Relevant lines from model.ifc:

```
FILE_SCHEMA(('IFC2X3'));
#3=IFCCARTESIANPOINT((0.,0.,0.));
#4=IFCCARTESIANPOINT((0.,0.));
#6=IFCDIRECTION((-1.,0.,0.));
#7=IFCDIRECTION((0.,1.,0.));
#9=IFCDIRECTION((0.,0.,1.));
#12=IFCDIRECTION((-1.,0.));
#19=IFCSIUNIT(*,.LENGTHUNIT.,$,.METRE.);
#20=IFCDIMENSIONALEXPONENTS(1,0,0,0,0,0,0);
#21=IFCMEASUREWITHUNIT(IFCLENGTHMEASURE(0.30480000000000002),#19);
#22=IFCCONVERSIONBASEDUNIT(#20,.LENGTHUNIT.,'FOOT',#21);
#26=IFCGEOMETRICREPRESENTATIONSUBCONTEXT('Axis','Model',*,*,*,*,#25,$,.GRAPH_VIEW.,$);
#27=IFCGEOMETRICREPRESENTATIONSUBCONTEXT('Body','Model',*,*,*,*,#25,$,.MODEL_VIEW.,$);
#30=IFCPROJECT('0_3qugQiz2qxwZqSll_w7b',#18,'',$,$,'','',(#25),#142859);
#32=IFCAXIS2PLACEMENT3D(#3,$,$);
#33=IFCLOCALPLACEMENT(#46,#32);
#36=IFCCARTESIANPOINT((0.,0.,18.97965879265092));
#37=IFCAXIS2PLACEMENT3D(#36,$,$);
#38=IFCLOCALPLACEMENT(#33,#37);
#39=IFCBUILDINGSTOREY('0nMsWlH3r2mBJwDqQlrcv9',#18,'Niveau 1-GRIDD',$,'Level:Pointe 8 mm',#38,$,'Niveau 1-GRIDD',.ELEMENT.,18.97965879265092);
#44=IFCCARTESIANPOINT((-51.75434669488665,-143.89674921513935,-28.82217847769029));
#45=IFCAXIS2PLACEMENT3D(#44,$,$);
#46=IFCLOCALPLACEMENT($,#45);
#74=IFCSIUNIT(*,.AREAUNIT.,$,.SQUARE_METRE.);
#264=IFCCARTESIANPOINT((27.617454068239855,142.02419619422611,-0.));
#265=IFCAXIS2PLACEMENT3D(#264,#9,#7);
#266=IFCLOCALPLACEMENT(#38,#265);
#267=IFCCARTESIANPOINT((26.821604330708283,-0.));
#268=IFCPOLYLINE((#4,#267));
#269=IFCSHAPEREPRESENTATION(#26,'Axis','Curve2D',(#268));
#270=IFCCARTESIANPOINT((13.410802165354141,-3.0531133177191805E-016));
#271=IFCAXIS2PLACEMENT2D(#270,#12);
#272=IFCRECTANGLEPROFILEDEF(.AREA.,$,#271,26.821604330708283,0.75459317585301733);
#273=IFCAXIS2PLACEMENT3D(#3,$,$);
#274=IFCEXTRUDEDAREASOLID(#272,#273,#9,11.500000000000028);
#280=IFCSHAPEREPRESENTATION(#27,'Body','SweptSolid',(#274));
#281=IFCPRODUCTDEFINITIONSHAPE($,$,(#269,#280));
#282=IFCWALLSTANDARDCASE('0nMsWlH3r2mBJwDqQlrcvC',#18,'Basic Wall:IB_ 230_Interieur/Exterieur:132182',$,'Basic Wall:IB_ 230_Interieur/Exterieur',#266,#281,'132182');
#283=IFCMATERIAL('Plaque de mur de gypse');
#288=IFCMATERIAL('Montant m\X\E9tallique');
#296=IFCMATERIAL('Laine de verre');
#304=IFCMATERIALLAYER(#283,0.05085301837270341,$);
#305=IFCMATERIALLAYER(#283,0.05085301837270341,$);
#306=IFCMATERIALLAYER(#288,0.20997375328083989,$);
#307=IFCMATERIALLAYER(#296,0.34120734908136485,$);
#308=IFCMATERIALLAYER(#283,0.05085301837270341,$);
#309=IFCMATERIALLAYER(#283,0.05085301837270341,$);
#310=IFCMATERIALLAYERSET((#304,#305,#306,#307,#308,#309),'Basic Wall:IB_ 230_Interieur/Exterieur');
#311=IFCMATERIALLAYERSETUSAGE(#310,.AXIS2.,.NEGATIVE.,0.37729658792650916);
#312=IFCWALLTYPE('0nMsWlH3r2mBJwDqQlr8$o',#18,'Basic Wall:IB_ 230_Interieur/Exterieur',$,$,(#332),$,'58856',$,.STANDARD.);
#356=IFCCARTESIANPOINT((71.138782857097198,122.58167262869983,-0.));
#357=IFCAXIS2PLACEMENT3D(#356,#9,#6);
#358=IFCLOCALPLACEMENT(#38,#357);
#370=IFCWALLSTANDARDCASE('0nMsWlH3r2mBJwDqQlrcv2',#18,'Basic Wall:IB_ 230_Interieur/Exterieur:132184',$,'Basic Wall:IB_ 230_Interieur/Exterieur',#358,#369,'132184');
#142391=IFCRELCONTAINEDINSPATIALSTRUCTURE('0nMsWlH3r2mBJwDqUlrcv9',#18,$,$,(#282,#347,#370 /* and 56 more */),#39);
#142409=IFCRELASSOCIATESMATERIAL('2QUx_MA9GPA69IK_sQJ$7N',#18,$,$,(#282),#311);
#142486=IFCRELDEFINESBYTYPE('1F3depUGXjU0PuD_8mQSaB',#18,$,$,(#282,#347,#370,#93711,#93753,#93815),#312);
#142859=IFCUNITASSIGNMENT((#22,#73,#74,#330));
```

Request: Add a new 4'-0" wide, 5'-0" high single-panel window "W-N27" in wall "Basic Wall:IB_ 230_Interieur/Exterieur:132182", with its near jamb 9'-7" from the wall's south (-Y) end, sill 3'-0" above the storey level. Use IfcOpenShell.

```python
import numpy as np
import ifcopenshell
import ifcopenshell.api.feature
import ifcopenshell.api.geometry
import ifcopenshell.api.root
import ifcopenshell.api.spatial
import ifcopenshell.api.type
import ifcopenshell.geom
import ifcopenshell.util.element
import ifcopenshell.util.placement
import ifcopenshell.util.representation
import ifcopenshell.util.shape
import ifcopenshell.util.unit

model = ifcopenshell.open("model.ifc")
unit_scale = ifcopenshell.util.unit.calculate_unit_scale(model)
settings = ifcopenshell.geom.settings()


def volume(element):
    """Net volume in cubic metres, openings subtracted."""
    shape = ifcopenshell.geom.create_shape(settings, element)
    return ifcopenshell.util.shape.get_volume(shape.geometry)


wall = model.by_id(282)
storey = ifcopenshell.util.element.get_container(wall, ifc_class="IfcBuildingStorey")
context = ifcopenshell.util.representation.get_context(model, "Model", "Body", "MODEL_VIEW")
before = volume(wall)

width, height, from_end, sill = 1.2192, 1.524, 2.921, 0.9144  # metres

# The wall runs along its own X axis, and the end named is its -X end.
wall_shape = ifcopenshell.geom.create_shape(settings, wall)
x, y, z = ifcopenshell.util.shape.get_vertices(wall_shape.geometry).T
start = x.min() + from_end
face, thickness = float(y.min()), float(y.max() - y.min())
wall_matrix = ifcopenshell.util.placement.get_local_placement(wall.ObjectPlacement)
level = ifcopenshell.util.placement.get_local_placement(storey.ObjectPlacement)[2, 3]


def in_wall(x, y):
    """Placement at x, y metres in the wall's axes, at sill height."""
    matrix = wall_matrix.copy()
    matrix[:, 3] = wall_matrix @ np.array([x / unit_scale, y / unit_scale, 0.0, 1.0])
    matrix[2, 3] = level + sill / unit_scale
    return matrix


# Opening: a box that overshoots both wall faces by 50 mm.
opening = ifcopenshell.api.root.create_entity(model, ifc_class="IfcOpeningElement")
box = ifcopenshell.api.geometry.add_wall_representation(
    model, context=context, length=width, height=height, thickness=thickness + 0.1
)
ifcopenshell.api.geometry.assign_representation(model, product=opening, representation=box)
ifcopenshell.api.geometry.edit_object_placement(model, product=opening, matrix=in_wall(start, face - 0.05), is_si=False)
ifcopenshell.api.feature.add_feature(model, feature=opening, element=wall)

window = ifcopenshell.api.root.create_entity(model, ifc_class="IfcWindow", name="W-N27")
window.OverallWidth, window.OverallHeight = width / unit_scale, height / unit_scale
body = ifcopenshell.api.geometry.add_window_representation(
    model,
    context=context,
    overall_width=window.OverallWidth,
    overall_height=window.OverallHeight,
    partition_type="SINGLE_PANEL",
)
ifcopenshell.api.geometry.assign_representation(model, product=window, representation=body)
ifcopenshell.api.spatial.assign_container(model, products=[window], relating_structure=storey)
fills = ifcopenshell.api.feature.add_filling(model, opening=opening, element=window)
fills.OwnerHistory = window.OwnerHistory  # required in IFC2X3

# IFC2X3 keeps the operation on the window style.
style = ifcopenshell.api.root.create_entity(model, ifc_class="IfcWindowStyle", name="W-N27")
style.OperationType, style.ConstructionType = "SINGLE_PANEL", "NOTDEFINED"
style.ParameterTakesPrecedence = style.Sizeable = False
ifcopenshell.api.type.assign_type(model, related_objects=[window], relating_type=style)

# Centre the window in the wall's thickness.
ifcopenshell.api.geometry.edit_object_placement(model, product=window, matrix=in_wall(start, face), is_si=False)
window_shape = ifcopenshell.geom.create_shape(settings, window)
depth = ifcopenshell.util.shape.get_vertices(window_shape.geometry)[:, 1]
offset = face + thickness / 2 - (depth.min() + depth.max()) / 2
ifcopenshell.api.geometry.edit_object_placement(model, product=window, matrix=in_wall(start, offset), is_si=False)

after = volume(wall)

print(f"wall volume {before:.3f} -> {after:.3f} m3")

model.write("model-out.ifc")
```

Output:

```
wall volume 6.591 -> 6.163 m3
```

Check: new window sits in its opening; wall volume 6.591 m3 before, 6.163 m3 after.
